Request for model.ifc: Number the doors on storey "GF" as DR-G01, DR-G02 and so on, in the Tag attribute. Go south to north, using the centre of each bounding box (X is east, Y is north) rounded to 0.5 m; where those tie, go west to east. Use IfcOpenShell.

First a look at what the model holds.

```python
import ifcopenshell
import ifcopenshell.util.element
import ifcopenshell.util.placement

model = ifcopenshell.open("model.ifc")
print(model.schema)
storey = next(s for s in model.by_type("IfcBuildingStorey") if s.Name == "GF")
doors = [e for e in ifcopenshell.util.element.get_decomposition(storey) if e.is_a("IfcDoor")]
for e in sorted(doors, key=lambda e: e.id()):
    origin = ifcopenshell.util.placement.get_local_placement(e.ObjectPlacement)[:3, 3]
    print(e.id(), e.Tag, e.Name, origin.round(2) + 0.0, sep=" | ")
```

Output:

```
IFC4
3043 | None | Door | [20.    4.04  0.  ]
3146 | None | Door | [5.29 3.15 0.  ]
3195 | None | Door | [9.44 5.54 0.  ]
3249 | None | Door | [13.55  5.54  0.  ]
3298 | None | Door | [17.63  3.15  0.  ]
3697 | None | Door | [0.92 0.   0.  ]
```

```python
import ifcopenshell
import ifcopenshell.geom
import ifcopenshell.util.element
import ifcopenshell.util.shape

model = ifcopenshell.open("model.ifc")
settings = ifcopenshell.geom.settings()
settings.set("use-world-coords", True)


def centre(element):
    shape = ifcopenshell.geom.create_shape(settings, element)
    return ifcopenshell.util.shape.get_bbox_centroid(shape.geometry)


storey = next(s for s in model.by_type("IfcBuildingStorey") if s.Name == "GF")
doors = [e for e in ifcopenshell.util.element.get_decomposition(storey) if e.is_a("IfcDoor")]

# Insertion points can sit at a corner or the storey origin, so sort by the geometry (in metres).
centres = {e: centre(e) for e in doors}
doors.sort(key=lambda e: (round(centres[e][1] / 0.5), centres[e][0]))

for i, e in enumerate(doors, start=1):
    number = f"DR-G{i:02d}"
    e.Tag = number
    print(e.id(), number)

model.write("model-out.ifc")
```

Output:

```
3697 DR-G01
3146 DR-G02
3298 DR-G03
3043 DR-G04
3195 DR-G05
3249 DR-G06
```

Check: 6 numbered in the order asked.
